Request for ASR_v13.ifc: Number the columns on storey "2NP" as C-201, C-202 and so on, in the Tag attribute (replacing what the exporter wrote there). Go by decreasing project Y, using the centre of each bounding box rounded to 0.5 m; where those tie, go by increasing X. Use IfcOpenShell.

First a look at what the model holds.

```python
import ifcopenshell
import ifcopenshell.util.element
import ifcopenshell.util.placement

model = ifcopenshell.open("ASR_v13.ifc")
print(model.schema)
storey = next(s for s in model.by_type("IfcBuildingStorey") if s.Name == "2NP")
columns = [e for e in ifcopenshell.util.element.get_decomposition(storey) if e.is_a("IfcColumn")]
for e in sorted(columns, key=lambda e: e.id()):
    origin = ifcopenshell.util.placement.get_local_placement(e.ObjectPlacement)[:3, 3]
    print(e.id(), e.Tag, e.Name, origin.round(2) + 0.0, sep=" | ")
```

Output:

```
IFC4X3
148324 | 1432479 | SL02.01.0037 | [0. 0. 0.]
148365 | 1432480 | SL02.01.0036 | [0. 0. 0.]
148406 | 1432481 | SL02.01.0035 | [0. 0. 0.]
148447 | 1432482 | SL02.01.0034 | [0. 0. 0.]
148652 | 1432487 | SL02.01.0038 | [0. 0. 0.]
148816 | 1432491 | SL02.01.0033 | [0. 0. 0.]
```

```python
import ifcopenshell
import ifcopenshell.geom
import ifcopenshell.util.element
import ifcopenshell.util.shape

model = ifcopenshell.open("ASR_v13.ifc")
settings = ifcopenshell.geom.settings()
settings.set("use-world-coords", True)


def centre(element):
    shape = ifcopenshell.geom.create_shape(settings, element)
    return ifcopenshell.util.shape.get_bbox_centroid(shape.geometry)


storey = next(s for s in model.by_type("IfcBuildingStorey") if s.Name == "2NP")
columns = [e for e in ifcopenshell.util.element.get_decomposition(storey) if e.is_a("IfcColumn")]

# Insertion points can sit at a corner or the storey origin, so sort by the geometry (in metres).
centres = {e: centre(e) for e in columns}
columns.sort(key=lambda e: (-round(centres[e][1] / 0.5), centres[e][0]))

for i, e in enumerate(columns, start=1):
    number = f"C-2{i:02d}"
    e.Tag = number
    print(e.id(), number)

model.write("ASR_v13_rev.ifc")
```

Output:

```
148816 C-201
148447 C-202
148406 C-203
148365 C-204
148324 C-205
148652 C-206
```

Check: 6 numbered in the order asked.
